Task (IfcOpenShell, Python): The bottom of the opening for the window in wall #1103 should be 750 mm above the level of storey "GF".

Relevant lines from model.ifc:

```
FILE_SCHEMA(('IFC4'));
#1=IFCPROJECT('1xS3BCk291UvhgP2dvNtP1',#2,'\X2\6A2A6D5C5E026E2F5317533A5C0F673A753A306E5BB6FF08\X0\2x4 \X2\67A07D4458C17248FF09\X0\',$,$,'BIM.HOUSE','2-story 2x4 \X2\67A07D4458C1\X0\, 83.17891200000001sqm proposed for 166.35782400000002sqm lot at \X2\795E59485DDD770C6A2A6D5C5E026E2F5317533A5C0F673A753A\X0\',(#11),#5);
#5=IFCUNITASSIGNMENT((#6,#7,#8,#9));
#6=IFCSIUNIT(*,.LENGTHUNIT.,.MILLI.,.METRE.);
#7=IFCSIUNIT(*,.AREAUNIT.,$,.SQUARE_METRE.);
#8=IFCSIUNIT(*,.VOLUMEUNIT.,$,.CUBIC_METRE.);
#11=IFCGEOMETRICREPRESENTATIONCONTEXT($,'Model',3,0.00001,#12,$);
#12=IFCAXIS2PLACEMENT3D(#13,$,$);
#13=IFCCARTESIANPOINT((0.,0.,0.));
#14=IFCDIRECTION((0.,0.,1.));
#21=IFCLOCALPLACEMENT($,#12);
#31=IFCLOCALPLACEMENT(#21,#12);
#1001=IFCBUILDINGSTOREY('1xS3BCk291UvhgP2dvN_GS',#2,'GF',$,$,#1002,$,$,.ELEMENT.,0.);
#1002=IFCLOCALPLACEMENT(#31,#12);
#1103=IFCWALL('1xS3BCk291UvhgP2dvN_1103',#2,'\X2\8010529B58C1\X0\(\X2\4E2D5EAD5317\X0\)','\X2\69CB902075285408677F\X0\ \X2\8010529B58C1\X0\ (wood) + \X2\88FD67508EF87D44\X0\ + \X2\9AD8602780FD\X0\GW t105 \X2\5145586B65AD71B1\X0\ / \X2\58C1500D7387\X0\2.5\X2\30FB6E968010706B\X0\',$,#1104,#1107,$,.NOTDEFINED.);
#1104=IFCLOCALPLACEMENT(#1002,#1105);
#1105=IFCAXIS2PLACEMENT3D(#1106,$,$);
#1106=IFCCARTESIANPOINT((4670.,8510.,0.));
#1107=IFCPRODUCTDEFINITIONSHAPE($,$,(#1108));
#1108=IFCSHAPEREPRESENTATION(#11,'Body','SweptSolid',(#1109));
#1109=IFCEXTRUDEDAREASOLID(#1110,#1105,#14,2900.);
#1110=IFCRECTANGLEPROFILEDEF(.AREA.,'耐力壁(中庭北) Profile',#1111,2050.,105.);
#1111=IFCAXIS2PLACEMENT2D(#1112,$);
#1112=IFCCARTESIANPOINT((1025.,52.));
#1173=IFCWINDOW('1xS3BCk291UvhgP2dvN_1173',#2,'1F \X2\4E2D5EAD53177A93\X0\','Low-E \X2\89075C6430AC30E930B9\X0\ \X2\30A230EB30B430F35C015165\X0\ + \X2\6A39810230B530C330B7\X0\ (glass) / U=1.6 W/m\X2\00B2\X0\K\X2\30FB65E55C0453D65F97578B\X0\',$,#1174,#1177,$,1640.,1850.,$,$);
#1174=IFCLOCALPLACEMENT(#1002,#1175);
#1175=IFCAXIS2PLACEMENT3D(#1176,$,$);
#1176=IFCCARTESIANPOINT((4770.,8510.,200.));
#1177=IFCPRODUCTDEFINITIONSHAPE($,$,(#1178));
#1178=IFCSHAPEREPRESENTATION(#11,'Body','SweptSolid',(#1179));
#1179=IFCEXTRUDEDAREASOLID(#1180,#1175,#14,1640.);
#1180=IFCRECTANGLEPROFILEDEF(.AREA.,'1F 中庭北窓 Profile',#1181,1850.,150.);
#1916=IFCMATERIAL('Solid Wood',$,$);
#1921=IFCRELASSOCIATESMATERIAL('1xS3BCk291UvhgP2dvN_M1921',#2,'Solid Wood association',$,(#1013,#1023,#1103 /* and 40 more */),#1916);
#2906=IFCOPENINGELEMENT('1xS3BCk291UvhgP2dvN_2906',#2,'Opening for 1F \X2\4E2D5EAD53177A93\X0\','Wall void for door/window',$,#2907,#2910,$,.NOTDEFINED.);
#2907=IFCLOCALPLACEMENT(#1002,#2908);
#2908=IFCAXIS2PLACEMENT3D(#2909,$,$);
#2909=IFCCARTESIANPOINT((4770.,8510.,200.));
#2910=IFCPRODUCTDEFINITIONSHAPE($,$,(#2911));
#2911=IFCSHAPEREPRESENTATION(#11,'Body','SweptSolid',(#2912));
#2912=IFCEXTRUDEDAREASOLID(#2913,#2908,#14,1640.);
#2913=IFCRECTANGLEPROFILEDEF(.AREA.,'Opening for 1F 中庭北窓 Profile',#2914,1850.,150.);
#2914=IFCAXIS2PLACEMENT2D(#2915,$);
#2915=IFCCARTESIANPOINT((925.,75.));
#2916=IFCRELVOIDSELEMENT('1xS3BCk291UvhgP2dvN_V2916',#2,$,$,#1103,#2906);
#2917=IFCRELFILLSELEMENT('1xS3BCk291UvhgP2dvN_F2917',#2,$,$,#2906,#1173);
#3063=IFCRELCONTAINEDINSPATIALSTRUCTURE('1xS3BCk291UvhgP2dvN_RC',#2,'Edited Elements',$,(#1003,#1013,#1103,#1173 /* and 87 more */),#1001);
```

```python
import numpy as np
import ifcopenshell
import ifcopenshell.api.geometry
import ifcopenshell.geom
import ifcopenshell.util.element
import ifcopenshell.util.placement
import ifcopenshell.util.shape
import ifcopenshell.util.unit

model = ifcopenshell.open("model.ifc")
unit_scale = ifcopenshell.util.unit.calculate_unit_scale(model)

window = model.by_guid("1xS3BCk291UvhgP2dvN_1173")
opening = window.FillsVoids[0].RelatingOpeningElement
storey = ifcopenshell.util.element.get_container(window, ifc_class="IfcBuildingStorey")
level = ifcopenshell.util.placement.get_local_placement(storey.ObjectPlacement)[2, 3]

# The opening's origin need not be at the sill, so measure its lowest point.
shape = ifcopenshell.geom.create_shape(ifcopenshell.geom.settings(), opening)
bottom = ifcopenshell.util.shape.get_shape_bottom_elevation(shape, shape.geometry) / unit_scale
dz = level + 0.75 / unit_scale - bottom

shift = np.array([0.0, 0.0, dz])
# The window is not placed relative to its opening, so move both.
for product in (opening, window):
    matrix = ifcopenshell.util.placement.get_local_placement(product.ObjectPlacement)
    matrix[:3, 3] += shift
    ifcopenshell.api.geometry.edit_object_placement(model, product=product, matrix=matrix, is_si=False)

print(f"moved by {dz * unit_scale:+.3f} m")

model.write("model_v2.ifc")
```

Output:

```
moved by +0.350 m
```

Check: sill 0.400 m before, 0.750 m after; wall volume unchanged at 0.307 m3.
